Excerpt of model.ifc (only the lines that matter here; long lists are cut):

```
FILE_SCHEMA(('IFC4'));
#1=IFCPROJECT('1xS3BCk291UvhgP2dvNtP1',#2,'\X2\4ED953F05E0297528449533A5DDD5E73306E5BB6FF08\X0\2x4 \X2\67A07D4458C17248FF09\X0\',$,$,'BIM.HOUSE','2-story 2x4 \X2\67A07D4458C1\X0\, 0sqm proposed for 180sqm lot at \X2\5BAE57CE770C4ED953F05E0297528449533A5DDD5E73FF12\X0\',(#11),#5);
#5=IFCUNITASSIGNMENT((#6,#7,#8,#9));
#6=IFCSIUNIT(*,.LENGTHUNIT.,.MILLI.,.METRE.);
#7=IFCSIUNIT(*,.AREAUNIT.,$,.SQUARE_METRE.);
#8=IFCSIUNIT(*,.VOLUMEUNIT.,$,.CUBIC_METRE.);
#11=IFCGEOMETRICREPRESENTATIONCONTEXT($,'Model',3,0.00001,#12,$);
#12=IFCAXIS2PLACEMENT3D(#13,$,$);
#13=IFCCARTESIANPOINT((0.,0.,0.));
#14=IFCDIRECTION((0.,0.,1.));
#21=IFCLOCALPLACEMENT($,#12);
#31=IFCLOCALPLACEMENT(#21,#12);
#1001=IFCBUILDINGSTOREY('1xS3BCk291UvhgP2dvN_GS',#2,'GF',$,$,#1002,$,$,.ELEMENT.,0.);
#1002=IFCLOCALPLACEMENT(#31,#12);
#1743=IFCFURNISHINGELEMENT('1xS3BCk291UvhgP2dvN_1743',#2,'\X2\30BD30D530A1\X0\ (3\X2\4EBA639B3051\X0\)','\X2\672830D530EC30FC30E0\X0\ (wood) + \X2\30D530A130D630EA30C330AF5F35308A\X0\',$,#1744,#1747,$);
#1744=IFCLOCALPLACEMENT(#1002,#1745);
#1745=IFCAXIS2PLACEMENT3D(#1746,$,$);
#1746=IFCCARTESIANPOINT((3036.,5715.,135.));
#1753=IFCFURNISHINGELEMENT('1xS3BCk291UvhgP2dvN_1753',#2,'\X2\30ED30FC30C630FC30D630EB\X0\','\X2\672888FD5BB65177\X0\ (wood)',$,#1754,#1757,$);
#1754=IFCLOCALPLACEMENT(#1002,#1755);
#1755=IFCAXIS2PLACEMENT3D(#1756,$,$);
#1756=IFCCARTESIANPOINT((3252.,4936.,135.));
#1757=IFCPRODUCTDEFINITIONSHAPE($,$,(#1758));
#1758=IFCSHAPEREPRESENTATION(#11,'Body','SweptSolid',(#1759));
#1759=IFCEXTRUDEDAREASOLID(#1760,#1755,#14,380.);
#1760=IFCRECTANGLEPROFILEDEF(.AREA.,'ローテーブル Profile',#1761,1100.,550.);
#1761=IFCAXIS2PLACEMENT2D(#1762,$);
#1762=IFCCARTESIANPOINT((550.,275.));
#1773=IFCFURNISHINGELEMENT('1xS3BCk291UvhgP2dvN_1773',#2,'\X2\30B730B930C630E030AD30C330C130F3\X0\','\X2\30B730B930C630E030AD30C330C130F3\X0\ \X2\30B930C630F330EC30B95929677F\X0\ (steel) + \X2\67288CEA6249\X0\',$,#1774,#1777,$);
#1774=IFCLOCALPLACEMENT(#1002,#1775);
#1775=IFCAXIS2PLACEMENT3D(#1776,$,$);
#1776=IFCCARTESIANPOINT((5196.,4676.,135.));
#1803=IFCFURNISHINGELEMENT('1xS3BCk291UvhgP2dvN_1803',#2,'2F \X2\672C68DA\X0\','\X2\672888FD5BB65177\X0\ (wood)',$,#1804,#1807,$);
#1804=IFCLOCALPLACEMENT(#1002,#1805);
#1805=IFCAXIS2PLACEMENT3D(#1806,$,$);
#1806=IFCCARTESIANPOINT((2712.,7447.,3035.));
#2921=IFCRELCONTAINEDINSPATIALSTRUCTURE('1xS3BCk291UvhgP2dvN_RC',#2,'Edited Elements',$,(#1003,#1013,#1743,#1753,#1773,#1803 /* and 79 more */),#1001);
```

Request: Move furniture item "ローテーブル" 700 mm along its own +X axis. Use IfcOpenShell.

```python
import ifcopenshell
import ifcopenshell.api.geometry
import ifcopenshell.util.placement
import ifcopenshell.util.unit

model = ifcopenshell.open("model.ifc")
unit_scale = ifcopenshell.util.unit.calculate_unit_scale(model)

item = model.by_id(1753)
matrix = ifcopenshell.util.placement.get_local_placement(item.ObjectPlacement)
matrix[:3, 3] += matrix[:3, 0] * 0.7 / unit_scale
ifcopenshell.api.geometry.edit_object_placement(model, product=item, matrix=matrix, is_si=False)

print(ifcopenshell.util.placement.get_local_placement(item.ObjectPlacement).round(3) + 0.0)

model.write("model-out.ifc")
```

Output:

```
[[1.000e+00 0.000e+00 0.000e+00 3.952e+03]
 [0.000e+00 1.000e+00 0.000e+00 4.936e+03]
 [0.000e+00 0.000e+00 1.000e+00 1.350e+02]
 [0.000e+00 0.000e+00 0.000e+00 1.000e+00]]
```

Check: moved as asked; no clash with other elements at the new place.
